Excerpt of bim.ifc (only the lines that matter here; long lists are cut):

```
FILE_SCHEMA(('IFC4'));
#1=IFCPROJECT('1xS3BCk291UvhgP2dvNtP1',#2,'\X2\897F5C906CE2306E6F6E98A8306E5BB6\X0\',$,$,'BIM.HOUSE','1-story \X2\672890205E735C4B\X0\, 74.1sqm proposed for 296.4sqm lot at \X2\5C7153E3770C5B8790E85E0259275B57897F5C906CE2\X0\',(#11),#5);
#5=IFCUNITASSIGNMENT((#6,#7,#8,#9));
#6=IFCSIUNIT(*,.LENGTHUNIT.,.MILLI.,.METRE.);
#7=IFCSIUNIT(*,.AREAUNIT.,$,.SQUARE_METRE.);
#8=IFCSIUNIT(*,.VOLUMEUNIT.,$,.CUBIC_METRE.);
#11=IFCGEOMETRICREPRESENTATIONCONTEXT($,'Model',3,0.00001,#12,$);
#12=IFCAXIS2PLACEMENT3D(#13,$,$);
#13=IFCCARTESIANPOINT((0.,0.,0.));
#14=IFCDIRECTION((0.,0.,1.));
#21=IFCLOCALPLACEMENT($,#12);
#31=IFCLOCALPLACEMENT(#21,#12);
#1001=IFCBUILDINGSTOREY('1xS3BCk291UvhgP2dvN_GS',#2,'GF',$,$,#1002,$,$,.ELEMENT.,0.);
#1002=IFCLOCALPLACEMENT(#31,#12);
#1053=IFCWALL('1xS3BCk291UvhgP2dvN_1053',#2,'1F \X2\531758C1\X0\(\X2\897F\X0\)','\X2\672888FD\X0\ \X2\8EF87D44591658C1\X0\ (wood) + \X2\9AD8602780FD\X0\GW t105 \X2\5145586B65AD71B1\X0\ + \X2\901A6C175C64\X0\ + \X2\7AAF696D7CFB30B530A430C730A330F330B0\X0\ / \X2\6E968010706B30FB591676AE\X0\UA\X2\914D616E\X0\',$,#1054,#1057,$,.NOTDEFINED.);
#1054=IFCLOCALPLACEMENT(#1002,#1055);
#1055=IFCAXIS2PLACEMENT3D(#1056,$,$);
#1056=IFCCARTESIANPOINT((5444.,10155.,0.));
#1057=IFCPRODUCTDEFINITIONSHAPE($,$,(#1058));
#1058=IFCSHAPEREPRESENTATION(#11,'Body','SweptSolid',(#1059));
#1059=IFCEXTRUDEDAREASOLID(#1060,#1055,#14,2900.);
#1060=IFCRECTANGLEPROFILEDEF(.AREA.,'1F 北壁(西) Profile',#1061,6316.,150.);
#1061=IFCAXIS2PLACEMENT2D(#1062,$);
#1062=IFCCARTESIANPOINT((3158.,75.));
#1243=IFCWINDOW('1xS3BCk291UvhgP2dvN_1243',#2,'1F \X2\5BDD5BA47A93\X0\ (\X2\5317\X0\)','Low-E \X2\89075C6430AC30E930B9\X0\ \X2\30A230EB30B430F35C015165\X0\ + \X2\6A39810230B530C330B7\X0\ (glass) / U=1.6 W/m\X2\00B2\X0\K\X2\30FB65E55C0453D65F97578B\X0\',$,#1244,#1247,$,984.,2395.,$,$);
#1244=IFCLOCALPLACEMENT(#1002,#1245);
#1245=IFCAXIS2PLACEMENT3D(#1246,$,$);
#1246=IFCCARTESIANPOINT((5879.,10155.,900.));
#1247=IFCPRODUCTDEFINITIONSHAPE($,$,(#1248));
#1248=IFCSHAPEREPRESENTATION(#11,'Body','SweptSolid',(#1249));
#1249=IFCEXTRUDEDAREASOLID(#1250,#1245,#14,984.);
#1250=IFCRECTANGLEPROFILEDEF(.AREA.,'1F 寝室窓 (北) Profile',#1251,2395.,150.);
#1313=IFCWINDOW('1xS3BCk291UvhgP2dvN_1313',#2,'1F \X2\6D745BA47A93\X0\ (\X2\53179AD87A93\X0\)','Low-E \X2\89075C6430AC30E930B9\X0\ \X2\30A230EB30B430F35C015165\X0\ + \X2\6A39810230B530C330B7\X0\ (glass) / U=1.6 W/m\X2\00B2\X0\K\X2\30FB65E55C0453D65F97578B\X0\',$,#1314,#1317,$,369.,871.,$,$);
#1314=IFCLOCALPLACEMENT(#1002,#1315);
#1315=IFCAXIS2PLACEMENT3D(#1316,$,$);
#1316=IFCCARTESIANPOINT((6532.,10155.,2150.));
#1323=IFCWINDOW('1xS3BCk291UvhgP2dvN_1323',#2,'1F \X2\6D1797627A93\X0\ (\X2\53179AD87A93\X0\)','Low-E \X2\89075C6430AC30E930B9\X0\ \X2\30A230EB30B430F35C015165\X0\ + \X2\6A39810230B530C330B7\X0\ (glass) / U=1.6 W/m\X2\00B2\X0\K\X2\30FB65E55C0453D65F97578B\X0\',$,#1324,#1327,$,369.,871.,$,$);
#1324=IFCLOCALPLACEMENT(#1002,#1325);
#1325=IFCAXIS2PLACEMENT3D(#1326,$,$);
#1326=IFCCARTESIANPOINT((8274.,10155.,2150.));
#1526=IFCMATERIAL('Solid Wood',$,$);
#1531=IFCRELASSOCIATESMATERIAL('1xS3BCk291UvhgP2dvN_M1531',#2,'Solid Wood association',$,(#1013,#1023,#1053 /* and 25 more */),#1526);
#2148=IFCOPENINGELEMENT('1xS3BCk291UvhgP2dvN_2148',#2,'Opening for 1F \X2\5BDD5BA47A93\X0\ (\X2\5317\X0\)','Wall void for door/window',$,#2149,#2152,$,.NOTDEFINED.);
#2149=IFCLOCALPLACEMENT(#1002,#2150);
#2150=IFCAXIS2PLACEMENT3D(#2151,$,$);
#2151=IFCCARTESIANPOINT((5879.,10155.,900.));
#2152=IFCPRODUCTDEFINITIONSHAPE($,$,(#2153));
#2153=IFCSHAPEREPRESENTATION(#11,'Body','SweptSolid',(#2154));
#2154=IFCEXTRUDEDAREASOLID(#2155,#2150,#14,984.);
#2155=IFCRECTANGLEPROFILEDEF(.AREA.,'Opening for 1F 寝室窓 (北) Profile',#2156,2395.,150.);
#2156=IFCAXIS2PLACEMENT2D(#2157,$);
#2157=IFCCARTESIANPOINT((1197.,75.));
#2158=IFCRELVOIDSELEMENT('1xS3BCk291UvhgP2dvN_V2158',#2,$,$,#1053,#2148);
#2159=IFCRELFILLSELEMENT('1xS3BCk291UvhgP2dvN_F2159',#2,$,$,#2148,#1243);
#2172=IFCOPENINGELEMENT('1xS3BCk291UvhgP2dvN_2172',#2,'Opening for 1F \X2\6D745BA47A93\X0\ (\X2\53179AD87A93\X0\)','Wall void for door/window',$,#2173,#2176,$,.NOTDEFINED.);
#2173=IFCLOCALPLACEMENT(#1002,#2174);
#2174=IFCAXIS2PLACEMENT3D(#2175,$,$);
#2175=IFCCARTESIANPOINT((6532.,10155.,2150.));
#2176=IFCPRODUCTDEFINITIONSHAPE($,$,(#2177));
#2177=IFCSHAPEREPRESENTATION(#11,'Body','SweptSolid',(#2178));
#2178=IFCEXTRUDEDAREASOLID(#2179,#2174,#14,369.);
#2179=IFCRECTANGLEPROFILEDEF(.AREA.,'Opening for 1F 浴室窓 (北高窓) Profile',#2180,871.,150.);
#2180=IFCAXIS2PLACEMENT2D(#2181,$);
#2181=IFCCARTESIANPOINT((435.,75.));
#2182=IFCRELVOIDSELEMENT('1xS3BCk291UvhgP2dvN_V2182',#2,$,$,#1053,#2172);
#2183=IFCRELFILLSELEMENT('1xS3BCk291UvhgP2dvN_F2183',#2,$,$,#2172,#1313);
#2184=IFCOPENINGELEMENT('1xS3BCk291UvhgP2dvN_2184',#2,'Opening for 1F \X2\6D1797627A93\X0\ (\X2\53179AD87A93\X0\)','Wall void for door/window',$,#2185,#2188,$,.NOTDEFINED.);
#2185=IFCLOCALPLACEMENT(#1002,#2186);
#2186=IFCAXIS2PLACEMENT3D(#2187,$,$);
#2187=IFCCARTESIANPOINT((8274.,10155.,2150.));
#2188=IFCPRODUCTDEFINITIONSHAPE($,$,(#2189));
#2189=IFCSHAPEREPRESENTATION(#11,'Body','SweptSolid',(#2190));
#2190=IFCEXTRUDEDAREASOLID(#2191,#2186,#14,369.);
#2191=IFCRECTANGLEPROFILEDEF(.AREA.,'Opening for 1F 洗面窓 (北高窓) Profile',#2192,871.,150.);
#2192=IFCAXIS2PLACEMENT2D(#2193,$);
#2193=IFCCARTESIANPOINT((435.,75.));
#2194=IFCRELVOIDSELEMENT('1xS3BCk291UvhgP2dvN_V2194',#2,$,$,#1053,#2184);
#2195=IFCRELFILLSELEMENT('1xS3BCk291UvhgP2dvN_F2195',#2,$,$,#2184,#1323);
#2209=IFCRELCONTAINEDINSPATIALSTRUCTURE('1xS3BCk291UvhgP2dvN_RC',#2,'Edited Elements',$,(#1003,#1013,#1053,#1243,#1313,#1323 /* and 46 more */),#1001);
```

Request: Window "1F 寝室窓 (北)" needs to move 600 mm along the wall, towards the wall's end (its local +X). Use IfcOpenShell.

```python
import ifcopenshell
import ifcopenshell.api.geometry
import ifcopenshell.util.placement
import ifcopenshell.util.unit

model = ifcopenshell.open("bim.ifc")
unit_scale = ifcopenshell.util.unit.calculate_unit_scale(model)

window = model.by_guid("1xS3BCk291UvhgP2dvN_1243")
opening = window.FillsVoids[0].RelatingOpeningElement
wall = opening.VoidsElements[0].RelatingBuildingElement

wall_matrix = ifcopenshell.util.placement.get_local_placement(wall.ObjectPlacement)
shift = wall_matrix[:3, 0] * 0.6 / unit_scale
before = ifcopenshell.util.placement.get_local_placement(window.ObjectPlacement)[:3, 3].copy()

# The window is not placed relative to its opening, so move both.
for product in (opening, window):
    matrix = ifcopenshell.util.placement.get_local_placement(product.ObjectPlacement)
    matrix[:3, 3] += shift
    ifcopenshell.api.geometry.edit_object_placement(model, product=product, matrix=matrix, is_si=False)

after = ifcopenshell.util.placement.get_local_placement(window.ObjectPlacement)[:3, 3]
print("window moved by", (after - before).round(3) + 0.0)

model.write("bim_v2.ifc")
```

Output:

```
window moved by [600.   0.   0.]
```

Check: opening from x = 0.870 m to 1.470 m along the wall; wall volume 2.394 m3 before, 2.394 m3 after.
